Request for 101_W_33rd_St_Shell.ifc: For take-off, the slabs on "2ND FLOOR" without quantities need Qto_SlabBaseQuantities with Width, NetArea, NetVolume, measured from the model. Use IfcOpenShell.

First a look at what the model holds.

```python
import ifcopenshell
import ifcopenshell.util.element
import ifcopenshell.util.unit

model = ifcopenshell.open("101_W_33rd_St_Shell.ifc")
print(model.schema)
for unit_type in ("LENGTHUNIT", "AREAUNIT", "VOLUMEUNIT"):
    print(unit_type, ifcopenshell.util.unit.calculate_unit_scale(model, unit_type))
storey = next(s for s in model.by_type("IfcBuildingStorey") if s.Name == "2ND FLOOR")
slabs = [e for e in ifcopenshell.util.element.get_decomposition(storey) if e.is_a("IfcSlab")]
for e in sorted(slabs, key=lambda e: e.id()):
    print(e.id(), e.is_a(), e.Name, list(ifcopenshell.util.element.get_psets(e, qtos_only=True)), sep=" | ")
```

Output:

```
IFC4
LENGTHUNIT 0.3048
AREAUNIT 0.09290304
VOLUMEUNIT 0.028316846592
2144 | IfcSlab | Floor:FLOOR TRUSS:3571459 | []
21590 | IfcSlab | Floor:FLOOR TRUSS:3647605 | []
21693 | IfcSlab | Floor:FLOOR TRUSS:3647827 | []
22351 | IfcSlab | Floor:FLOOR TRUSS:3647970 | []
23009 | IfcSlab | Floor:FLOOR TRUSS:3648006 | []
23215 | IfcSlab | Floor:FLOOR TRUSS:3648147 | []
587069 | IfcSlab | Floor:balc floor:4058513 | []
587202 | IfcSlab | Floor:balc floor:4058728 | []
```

```python
import ifcopenshell
import ifcopenshell.api.pset
import ifcopenshell.geom
import ifcopenshell.util.element
import ifcopenshell.util.shape
import ifcopenshell.util.unit

model = ifcopenshell.open("101_W_33rd_St_Shell.ifc")
unit_scale = ifcopenshell.util.unit.calculate_unit_scale(model)
area_scale = ifcopenshell.util.unit.calculate_unit_scale(model, "AREAUNIT")
volume_scale = ifcopenshell.util.unit.calculate_unit_scale(model, "VOLUMEUNIT")
settings = ifcopenshell.geom.settings()

storey = next(s for s in model.by_type("IfcBuildingStorey") if s.Name == "2ND FLOOR")
slabs = [e for e in ifcopenshell.util.element.get_decomposition(storey) if e.is_a("IfcSlab")]

for e in sorted(slabs, key=lambda e: e.id()):
    if ifcopenshell.util.element.get_psets(e, qtos_only=True, should_inherit=False):
        continue
    # Geometry comes back in metres, in the element's own axes.
    shape = ifcopenshell.geom.create_shape(settings, e)
    values = {
        "Width": ifcopenshell.util.shape.get_z(shape.geometry) / unit_scale,
        "NetArea": ifcopenshell.util.shape.get_footprint_area(shape.geometry) / area_scale,
        "NetVolume": ifcopenshell.util.shape.get_volume(shape.geometry) / volume_scale,
    }
    qto = ifcopenshell.api.pset.add_qto(model, product=e, name="Qto_SlabBaseQuantities")
    ifcopenshell.api.pset.edit_qto(model, qto=qto, properties=values)
    print(e.id(), {k: round(v, 3) for k, v in values.items()})

model.write("101_W_33rd_St_Shell_updated.ifc")
```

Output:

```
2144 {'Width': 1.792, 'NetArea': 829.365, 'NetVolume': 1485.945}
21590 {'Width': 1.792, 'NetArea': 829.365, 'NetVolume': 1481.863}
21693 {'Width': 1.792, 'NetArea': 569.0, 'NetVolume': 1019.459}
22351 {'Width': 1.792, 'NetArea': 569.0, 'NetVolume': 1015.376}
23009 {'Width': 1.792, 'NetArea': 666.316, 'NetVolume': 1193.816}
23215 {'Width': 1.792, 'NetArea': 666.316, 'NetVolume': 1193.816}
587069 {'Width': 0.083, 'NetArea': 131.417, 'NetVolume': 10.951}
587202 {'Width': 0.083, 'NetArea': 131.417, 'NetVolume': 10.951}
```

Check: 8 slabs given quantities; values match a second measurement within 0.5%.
